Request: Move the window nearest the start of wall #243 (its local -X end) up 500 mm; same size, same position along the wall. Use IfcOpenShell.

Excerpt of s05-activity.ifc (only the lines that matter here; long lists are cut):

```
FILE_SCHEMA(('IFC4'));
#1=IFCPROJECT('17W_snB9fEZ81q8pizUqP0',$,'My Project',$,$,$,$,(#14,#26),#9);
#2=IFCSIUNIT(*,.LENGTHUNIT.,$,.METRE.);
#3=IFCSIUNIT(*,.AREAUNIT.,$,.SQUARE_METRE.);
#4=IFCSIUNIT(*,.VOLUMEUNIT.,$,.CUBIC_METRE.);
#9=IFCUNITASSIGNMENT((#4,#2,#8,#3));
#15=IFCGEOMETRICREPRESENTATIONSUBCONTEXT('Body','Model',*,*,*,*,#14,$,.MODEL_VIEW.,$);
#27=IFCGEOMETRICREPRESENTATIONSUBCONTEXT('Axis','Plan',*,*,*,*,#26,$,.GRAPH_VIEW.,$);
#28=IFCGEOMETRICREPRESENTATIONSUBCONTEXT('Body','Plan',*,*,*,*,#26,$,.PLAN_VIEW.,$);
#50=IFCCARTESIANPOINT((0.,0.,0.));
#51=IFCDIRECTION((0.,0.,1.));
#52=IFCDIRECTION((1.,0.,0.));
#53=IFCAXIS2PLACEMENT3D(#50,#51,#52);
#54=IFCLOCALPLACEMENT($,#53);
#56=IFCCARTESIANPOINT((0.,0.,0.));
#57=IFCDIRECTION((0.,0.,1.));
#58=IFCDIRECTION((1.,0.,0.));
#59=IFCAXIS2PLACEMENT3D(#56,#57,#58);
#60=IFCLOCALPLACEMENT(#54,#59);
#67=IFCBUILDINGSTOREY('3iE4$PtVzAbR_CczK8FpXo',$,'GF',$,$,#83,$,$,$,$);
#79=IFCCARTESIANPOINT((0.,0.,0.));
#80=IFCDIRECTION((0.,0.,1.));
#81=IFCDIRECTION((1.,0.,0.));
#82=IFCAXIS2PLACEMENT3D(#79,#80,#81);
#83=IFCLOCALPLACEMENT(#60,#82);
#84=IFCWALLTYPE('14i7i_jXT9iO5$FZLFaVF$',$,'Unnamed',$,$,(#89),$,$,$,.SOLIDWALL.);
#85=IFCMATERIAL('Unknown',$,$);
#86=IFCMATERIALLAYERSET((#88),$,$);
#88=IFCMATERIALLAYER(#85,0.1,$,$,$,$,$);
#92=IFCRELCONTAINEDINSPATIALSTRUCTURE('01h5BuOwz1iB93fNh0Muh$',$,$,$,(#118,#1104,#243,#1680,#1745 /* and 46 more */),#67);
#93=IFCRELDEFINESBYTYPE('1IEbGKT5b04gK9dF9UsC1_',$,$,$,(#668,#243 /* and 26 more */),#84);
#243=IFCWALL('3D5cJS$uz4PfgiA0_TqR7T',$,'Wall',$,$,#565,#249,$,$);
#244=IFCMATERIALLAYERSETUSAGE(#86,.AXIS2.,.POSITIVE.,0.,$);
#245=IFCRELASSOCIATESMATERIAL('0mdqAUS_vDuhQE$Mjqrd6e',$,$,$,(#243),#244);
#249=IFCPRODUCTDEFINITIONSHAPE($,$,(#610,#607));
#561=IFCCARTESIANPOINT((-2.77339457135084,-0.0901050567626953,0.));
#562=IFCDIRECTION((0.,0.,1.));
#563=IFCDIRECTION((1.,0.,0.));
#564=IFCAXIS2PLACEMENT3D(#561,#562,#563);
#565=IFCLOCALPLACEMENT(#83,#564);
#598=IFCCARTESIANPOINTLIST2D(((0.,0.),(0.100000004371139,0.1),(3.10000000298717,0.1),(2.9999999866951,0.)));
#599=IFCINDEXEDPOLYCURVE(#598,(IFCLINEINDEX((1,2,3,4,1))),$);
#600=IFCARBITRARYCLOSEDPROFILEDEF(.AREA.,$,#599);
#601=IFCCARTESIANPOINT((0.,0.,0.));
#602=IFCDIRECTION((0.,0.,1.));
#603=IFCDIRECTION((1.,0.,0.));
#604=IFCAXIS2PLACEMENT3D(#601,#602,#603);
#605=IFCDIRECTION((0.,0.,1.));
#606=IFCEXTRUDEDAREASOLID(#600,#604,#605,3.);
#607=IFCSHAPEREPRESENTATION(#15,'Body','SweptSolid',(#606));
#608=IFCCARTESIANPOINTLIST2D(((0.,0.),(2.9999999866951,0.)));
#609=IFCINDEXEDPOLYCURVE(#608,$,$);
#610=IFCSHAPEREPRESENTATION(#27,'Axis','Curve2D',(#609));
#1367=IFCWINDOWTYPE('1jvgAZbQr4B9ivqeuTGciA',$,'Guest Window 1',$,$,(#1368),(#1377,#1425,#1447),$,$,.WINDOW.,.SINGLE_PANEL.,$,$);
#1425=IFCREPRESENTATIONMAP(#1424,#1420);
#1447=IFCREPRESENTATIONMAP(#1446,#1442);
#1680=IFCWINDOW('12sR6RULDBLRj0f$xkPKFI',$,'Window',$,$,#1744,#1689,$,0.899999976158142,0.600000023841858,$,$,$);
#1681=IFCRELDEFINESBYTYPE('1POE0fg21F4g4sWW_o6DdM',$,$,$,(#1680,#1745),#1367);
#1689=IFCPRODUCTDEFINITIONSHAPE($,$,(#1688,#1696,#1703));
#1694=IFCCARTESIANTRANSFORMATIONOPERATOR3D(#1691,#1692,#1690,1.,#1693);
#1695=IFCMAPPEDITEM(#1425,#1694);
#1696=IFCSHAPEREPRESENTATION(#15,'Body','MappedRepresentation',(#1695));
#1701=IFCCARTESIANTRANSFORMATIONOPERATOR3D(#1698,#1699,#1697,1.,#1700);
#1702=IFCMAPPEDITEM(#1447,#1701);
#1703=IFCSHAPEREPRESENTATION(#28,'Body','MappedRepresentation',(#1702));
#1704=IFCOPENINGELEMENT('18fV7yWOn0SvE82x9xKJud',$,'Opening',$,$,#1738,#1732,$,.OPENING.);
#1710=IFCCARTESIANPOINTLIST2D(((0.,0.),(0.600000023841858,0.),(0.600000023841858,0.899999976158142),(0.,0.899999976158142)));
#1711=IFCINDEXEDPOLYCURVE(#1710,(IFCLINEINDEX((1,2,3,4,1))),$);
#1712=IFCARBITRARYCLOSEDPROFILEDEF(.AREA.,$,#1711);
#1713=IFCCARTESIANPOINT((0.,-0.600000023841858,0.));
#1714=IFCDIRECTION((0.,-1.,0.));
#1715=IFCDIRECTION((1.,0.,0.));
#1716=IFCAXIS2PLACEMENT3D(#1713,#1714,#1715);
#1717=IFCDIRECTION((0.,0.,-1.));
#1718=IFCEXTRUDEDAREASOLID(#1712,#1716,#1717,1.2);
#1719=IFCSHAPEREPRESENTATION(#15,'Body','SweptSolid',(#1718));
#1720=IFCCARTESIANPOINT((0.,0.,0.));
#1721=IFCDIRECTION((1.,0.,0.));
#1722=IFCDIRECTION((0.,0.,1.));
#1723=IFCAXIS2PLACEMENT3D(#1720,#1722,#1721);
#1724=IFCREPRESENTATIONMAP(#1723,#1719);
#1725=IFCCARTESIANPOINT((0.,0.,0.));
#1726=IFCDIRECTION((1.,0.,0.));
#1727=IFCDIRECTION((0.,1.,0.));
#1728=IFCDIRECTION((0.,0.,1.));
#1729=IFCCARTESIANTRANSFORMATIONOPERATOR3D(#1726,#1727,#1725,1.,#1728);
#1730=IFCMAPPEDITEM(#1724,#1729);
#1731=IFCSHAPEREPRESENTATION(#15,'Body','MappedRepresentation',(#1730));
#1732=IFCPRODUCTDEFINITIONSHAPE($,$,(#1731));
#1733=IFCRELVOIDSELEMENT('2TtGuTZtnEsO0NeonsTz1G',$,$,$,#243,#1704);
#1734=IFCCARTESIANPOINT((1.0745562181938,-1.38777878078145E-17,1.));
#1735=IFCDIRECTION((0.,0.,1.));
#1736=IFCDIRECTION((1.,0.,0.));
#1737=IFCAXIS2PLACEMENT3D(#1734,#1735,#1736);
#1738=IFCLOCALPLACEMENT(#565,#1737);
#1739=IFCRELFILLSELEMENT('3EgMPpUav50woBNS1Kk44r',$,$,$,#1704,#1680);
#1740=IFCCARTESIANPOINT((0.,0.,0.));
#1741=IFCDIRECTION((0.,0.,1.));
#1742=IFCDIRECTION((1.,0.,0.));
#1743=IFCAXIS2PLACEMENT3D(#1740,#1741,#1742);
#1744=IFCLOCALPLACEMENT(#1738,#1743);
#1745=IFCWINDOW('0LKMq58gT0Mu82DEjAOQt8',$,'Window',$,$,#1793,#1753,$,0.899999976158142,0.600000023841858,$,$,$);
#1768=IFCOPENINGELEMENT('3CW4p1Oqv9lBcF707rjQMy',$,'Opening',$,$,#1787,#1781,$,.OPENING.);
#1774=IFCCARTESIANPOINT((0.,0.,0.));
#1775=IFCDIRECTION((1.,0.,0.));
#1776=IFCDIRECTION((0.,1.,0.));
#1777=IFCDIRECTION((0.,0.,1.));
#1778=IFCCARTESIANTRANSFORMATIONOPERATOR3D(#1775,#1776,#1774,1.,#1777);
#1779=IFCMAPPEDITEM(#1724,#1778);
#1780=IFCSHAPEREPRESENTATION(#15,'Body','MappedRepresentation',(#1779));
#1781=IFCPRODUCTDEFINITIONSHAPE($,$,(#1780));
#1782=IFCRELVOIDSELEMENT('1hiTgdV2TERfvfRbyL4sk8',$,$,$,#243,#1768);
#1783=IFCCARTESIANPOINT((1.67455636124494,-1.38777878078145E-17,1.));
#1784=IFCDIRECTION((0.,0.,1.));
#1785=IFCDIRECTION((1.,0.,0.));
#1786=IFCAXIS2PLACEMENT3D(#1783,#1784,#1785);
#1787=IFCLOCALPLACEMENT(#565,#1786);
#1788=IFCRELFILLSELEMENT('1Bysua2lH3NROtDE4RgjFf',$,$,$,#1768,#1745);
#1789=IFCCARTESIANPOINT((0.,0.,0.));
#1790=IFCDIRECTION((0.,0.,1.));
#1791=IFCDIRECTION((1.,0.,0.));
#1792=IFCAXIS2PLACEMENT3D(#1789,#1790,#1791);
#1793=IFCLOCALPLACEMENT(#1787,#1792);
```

```python
import numpy as np
import ifcopenshell
import ifcopenshell.api.geometry
import ifcopenshell.util.placement
import ifcopenshell.util.unit

model = ifcopenshell.open("s05-activity.ifc")
unit_scale = ifcopenshell.util.unit.calculate_unit_scale(model)

window = model.by_id(1680)
opening = window.FillsVoids[0].RelatingOpeningElement
dz = 0.5

shift = np.array([0.0, 0.0, dz])
# The window is placed relative to its opening, so it follows when the opening moves.
matrix = ifcopenshell.util.placement.get_local_placement(opening.ObjectPlacement)
matrix[:3, 3] += shift
ifcopenshell.api.geometry.edit_object_placement(
    model, product=opening, matrix=matrix, is_si=False, should_transform_children=True
)

print(f"moved by {dz * unit_scale:+.3f} m")

model.write("s05-activity_v2.ifc")
```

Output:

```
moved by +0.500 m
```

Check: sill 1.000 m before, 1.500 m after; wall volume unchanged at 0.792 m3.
